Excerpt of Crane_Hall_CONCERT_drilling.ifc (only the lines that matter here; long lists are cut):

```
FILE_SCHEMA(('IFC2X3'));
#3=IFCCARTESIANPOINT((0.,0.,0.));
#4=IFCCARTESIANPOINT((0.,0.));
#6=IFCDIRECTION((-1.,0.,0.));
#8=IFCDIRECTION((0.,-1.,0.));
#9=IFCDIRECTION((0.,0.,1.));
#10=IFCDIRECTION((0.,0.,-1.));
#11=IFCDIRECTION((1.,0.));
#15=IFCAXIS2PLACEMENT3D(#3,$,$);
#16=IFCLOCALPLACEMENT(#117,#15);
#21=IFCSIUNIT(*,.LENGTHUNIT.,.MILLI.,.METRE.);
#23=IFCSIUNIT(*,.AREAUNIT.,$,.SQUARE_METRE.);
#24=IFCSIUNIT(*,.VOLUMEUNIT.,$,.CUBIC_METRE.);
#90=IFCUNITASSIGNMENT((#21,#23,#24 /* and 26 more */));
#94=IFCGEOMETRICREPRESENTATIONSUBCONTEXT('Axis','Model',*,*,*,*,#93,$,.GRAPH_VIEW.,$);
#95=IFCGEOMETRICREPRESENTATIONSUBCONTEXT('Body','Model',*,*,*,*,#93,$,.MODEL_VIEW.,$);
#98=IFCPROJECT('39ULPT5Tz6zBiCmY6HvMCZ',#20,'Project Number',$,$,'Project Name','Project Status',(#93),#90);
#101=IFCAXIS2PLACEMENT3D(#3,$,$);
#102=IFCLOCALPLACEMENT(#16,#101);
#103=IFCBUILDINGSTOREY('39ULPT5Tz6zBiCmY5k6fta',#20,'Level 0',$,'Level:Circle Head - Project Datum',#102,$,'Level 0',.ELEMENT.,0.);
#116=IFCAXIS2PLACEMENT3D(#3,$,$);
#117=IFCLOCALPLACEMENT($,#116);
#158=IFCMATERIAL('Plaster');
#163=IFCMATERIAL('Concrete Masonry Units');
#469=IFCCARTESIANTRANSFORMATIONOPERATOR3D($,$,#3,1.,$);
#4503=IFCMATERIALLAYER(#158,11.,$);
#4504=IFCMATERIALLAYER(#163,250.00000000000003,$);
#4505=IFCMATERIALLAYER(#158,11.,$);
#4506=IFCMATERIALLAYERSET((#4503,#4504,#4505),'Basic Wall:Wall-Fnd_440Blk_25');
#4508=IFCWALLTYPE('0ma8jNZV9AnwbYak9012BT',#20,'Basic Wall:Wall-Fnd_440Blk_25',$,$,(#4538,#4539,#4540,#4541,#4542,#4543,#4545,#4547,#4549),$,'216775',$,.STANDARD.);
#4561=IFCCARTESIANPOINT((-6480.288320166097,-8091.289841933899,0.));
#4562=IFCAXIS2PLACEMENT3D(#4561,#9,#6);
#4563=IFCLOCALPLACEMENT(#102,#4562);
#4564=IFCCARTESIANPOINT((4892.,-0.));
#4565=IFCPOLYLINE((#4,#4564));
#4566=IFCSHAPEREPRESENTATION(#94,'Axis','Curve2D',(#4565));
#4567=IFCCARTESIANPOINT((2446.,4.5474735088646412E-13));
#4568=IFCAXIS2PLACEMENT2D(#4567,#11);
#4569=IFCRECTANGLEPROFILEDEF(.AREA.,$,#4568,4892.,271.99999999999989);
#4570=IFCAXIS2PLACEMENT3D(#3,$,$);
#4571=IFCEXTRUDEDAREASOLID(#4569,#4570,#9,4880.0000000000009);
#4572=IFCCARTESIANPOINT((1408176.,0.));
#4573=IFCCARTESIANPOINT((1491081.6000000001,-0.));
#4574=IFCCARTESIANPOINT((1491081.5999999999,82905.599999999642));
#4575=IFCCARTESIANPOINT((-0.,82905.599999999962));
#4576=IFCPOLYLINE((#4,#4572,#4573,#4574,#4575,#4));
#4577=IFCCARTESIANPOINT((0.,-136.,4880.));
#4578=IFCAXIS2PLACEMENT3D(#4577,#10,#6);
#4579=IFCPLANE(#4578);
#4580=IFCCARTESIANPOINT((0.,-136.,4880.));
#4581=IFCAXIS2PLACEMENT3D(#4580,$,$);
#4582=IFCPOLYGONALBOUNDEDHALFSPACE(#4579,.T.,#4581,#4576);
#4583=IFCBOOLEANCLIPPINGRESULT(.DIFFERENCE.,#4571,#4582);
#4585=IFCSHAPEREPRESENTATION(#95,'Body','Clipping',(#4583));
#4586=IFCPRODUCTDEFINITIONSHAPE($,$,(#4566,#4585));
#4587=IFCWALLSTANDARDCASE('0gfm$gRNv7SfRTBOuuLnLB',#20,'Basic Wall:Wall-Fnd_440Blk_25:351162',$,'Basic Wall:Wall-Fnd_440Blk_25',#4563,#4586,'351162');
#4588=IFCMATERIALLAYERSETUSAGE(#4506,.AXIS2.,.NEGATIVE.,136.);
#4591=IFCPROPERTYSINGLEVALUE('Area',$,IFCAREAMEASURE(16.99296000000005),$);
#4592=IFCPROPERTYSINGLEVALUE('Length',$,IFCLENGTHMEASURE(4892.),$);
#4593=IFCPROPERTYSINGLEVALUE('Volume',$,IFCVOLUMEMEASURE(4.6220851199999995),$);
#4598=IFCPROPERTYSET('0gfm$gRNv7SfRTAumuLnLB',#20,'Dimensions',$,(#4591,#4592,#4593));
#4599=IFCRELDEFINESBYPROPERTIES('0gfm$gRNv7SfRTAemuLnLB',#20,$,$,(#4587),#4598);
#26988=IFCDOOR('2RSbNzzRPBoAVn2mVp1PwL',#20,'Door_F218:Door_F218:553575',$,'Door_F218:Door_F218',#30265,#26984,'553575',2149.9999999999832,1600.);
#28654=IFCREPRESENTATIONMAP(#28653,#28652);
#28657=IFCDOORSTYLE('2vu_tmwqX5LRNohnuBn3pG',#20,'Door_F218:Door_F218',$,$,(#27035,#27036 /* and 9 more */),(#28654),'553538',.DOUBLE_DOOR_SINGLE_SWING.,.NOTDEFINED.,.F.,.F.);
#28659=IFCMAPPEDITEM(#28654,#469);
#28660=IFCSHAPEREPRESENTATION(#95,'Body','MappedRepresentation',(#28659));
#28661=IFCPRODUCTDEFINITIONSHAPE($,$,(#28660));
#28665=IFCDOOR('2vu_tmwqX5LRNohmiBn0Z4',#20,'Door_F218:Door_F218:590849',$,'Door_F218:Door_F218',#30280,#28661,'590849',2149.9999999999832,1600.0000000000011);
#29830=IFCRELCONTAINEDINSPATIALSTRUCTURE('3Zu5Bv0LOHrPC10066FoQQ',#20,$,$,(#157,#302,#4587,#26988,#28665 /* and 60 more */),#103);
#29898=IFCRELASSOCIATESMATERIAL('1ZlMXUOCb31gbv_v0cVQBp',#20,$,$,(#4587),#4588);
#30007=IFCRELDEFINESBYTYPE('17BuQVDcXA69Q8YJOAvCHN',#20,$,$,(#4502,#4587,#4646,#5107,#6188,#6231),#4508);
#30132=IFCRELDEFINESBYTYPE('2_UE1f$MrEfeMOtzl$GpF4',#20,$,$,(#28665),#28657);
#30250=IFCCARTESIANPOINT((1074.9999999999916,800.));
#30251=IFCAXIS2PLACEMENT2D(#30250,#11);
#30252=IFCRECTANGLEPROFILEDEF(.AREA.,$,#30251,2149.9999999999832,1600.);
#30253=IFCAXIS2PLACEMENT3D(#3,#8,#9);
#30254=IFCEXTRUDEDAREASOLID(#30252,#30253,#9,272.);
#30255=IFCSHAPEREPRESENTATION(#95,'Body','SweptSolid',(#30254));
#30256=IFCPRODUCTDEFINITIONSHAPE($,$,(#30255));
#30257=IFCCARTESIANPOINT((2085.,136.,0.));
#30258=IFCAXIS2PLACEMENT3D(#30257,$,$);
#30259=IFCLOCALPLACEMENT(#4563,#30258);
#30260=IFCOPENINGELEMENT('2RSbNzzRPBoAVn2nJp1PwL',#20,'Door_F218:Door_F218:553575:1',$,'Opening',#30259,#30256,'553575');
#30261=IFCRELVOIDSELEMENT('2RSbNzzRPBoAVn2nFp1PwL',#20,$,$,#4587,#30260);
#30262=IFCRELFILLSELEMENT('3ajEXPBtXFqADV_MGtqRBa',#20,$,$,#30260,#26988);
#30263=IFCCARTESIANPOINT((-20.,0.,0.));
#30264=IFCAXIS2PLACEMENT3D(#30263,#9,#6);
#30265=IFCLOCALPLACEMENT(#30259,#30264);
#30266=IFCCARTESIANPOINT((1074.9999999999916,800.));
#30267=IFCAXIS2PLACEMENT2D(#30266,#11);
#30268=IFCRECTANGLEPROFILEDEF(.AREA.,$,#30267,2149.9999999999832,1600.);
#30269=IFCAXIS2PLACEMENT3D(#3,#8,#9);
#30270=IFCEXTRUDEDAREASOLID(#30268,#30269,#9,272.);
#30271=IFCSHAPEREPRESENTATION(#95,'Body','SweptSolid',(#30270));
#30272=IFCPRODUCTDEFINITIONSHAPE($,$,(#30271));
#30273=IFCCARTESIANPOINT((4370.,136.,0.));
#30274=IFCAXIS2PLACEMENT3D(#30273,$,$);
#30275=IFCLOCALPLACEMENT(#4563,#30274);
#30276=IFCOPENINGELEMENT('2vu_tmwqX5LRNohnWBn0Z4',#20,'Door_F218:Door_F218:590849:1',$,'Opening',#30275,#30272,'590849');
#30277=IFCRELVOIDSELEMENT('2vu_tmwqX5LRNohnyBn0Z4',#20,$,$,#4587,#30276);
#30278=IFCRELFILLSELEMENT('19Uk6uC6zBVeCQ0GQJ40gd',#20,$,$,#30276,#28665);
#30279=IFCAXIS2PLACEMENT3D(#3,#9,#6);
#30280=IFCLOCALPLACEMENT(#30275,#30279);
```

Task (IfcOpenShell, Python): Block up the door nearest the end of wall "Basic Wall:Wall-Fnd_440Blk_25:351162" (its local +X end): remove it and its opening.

```python
import ifcopenshell
import ifcopenshell.api.feature
import ifcopenshell.api.pset
import ifcopenshell.api.root
import ifcopenshell.geom
import ifcopenshell.util.element
import ifcopenshell.util.shape
import ifcopenshell.util.unit

model = ifcopenshell.open("Crane_Hall_CONCERT_drilling.ifc")
area_scale = ifcopenshell.util.unit.calculate_unit_scale(model, "AREAUNIT")
volume_scale = ifcopenshell.util.unit.calculate_unit_scale(model, "VOLUMEUNIT")
settings = ifcopenshell.geom.settings()


def volume(element):
    """Net volume in cubic metres, openings subtracted."""
    shape = ifcopenshell.geom.create_shape(settings, element)
    return ifcopenshell.util.shape.get_volume(shape.geometry)


door = model.by_guid("2vu_tmwqX5LRNohmiBn0Z4")
opening = door.FillsVoids[0].RelatingOpeningElement
wall = opening.VoidsElements[0].RelatingBuildingElement
before = volume(wall)

ifcopenshell.api.root.remove_product(model, product=door)
ifcopenshell.api.feature.remove_feature(model, feature=opening)

after = volume(wall)
thickness = 0.272  # wall thickness in metres

# Update the wall's stored quantities.
pset = model.by_id(ifcopenshell.util.element.get_pset(wall, "Dimensions", should_inherit=False)["id"])
ifcopenshell.api.pset.edit_pset(model, pset=pset, properties={
    "Area": model.create_entity("IfcAreaMeasure", after / thickness / area_scale),
    "Volume": model.create_entity("IfcVolumeMeasure", after / volume_scale),
})

print(f"wall volume {before:.3f} -> {after:.3f} m3")

model.write("Crane_Hall_CONCERT_drilling-out.ifc")
```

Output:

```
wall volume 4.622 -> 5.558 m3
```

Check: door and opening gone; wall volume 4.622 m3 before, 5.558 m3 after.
